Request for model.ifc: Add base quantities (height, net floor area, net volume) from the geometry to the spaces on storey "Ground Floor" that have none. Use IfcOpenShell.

First a look at what the model holds.

```python
import ifcopenshell
import ifcopenshell.util.element
import ifcopenshell.util.unit

model = ifcopenshell.open("model.ifc")
print(model.schema)
for unit_type in ("LENGTHUNIT", "AREAUNIT", "VOLUMEUNIT"):
    print(unit_type, ifcopenshell.util.unit.calculate_unit_scale(model, unit_type))
storey = next(s for s in model.by_type("IfcBuildingStorey") if s.Name == "Ground Floor")
spaces = [e for e in ifcopenshell.util.element.get_decomposition(storey) if e.is_a("IfcSpace")]
for e in sorted(spaces, key=lambda e: e.id()):
    print(e.id(), e.is_a(), e.Name, list(ifcopenshell.util.element.get_psets(e, qtos_only=True)), sep=" | ")
```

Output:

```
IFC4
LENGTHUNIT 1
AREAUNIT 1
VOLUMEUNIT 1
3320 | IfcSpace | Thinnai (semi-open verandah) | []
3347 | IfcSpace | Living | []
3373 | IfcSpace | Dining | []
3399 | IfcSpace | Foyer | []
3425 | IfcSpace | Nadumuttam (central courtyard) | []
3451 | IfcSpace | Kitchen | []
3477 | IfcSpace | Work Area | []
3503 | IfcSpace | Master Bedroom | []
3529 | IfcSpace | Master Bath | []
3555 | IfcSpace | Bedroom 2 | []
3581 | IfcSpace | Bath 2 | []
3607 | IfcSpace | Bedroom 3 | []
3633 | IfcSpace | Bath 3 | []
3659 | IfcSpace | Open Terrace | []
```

```python
import ifcopenshell
import ifcopenshell.api.pset
import ifcopenshell.geom
import ifcopenshell.util.element
import ifcopenshell.util.shape
import ifcopenshell.util.unit

model = ifcopenshell.open("model.ifc")
unit_scale = ifcopenshell.util.unit.calculate_unit_scale(model)
area_scale = ifcopenshell.util.unit.calculate_unit_scale(model, "AREAUNIT")
volume_scale = ifcopenshell.util.unit.calculate_unit_scale(model, "VOLUMEUNIT")
settings = ifcopenshell.geom.settings()

storey = next(s for s in model.by_type("IfcBuildingStorey") if s.Name == "Ground Floor")
spaces = [e for e in ifcopenshell.util.element.get_decomposition(storey) if e.is_a("IfcSpace")]

for e in sorted(spaces, key=lambda e: e.id()):
    if ifcopenshell.util.element.get_psets(e, qtos_only=True, should_inherit=False):
        continue
    # Geometry comes back in metres, in the element's own axes.
    shape = ifcopenshell.geom.create_shape(settings, e)
    values = {
        "Height": ifcopenshell.util.shape.get_z(shape.geometry) / unit_scale,
        "NetFloorArea": ifcopenshell.util.shape.get_footprint_area(shape.geometry) / area_scale,
        "NetVolume": ifcopenshell.util.shape.get_volume(shape.geometry) / volume_scale,
    }
    qto = ifcopenshell.api.pset.add_qto(model, product=e, name="Qto_SpaceBaseQuantities")
    ifcopenshell.api.pset.edit_qto(model, qto=qto, properties=values)
    print(e.id(), {k: round(v, 3) for k, v in values.items()})

model.write("model-out.ifc")
```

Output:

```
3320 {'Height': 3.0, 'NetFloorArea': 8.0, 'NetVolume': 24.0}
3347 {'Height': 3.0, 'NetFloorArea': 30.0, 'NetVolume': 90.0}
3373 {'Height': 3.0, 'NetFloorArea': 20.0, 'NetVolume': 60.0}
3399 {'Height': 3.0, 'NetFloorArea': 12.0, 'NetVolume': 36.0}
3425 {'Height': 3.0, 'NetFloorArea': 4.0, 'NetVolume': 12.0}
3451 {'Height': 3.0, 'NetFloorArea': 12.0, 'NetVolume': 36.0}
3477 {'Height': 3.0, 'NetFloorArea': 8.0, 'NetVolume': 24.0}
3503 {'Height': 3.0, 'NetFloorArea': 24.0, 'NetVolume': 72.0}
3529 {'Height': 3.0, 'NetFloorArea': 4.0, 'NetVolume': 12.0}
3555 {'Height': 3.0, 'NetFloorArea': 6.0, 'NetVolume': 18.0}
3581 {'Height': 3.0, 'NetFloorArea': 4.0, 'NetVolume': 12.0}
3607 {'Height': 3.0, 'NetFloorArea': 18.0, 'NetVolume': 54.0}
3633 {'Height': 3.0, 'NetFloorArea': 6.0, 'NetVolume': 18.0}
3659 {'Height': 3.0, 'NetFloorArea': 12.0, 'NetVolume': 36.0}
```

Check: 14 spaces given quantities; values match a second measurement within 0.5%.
